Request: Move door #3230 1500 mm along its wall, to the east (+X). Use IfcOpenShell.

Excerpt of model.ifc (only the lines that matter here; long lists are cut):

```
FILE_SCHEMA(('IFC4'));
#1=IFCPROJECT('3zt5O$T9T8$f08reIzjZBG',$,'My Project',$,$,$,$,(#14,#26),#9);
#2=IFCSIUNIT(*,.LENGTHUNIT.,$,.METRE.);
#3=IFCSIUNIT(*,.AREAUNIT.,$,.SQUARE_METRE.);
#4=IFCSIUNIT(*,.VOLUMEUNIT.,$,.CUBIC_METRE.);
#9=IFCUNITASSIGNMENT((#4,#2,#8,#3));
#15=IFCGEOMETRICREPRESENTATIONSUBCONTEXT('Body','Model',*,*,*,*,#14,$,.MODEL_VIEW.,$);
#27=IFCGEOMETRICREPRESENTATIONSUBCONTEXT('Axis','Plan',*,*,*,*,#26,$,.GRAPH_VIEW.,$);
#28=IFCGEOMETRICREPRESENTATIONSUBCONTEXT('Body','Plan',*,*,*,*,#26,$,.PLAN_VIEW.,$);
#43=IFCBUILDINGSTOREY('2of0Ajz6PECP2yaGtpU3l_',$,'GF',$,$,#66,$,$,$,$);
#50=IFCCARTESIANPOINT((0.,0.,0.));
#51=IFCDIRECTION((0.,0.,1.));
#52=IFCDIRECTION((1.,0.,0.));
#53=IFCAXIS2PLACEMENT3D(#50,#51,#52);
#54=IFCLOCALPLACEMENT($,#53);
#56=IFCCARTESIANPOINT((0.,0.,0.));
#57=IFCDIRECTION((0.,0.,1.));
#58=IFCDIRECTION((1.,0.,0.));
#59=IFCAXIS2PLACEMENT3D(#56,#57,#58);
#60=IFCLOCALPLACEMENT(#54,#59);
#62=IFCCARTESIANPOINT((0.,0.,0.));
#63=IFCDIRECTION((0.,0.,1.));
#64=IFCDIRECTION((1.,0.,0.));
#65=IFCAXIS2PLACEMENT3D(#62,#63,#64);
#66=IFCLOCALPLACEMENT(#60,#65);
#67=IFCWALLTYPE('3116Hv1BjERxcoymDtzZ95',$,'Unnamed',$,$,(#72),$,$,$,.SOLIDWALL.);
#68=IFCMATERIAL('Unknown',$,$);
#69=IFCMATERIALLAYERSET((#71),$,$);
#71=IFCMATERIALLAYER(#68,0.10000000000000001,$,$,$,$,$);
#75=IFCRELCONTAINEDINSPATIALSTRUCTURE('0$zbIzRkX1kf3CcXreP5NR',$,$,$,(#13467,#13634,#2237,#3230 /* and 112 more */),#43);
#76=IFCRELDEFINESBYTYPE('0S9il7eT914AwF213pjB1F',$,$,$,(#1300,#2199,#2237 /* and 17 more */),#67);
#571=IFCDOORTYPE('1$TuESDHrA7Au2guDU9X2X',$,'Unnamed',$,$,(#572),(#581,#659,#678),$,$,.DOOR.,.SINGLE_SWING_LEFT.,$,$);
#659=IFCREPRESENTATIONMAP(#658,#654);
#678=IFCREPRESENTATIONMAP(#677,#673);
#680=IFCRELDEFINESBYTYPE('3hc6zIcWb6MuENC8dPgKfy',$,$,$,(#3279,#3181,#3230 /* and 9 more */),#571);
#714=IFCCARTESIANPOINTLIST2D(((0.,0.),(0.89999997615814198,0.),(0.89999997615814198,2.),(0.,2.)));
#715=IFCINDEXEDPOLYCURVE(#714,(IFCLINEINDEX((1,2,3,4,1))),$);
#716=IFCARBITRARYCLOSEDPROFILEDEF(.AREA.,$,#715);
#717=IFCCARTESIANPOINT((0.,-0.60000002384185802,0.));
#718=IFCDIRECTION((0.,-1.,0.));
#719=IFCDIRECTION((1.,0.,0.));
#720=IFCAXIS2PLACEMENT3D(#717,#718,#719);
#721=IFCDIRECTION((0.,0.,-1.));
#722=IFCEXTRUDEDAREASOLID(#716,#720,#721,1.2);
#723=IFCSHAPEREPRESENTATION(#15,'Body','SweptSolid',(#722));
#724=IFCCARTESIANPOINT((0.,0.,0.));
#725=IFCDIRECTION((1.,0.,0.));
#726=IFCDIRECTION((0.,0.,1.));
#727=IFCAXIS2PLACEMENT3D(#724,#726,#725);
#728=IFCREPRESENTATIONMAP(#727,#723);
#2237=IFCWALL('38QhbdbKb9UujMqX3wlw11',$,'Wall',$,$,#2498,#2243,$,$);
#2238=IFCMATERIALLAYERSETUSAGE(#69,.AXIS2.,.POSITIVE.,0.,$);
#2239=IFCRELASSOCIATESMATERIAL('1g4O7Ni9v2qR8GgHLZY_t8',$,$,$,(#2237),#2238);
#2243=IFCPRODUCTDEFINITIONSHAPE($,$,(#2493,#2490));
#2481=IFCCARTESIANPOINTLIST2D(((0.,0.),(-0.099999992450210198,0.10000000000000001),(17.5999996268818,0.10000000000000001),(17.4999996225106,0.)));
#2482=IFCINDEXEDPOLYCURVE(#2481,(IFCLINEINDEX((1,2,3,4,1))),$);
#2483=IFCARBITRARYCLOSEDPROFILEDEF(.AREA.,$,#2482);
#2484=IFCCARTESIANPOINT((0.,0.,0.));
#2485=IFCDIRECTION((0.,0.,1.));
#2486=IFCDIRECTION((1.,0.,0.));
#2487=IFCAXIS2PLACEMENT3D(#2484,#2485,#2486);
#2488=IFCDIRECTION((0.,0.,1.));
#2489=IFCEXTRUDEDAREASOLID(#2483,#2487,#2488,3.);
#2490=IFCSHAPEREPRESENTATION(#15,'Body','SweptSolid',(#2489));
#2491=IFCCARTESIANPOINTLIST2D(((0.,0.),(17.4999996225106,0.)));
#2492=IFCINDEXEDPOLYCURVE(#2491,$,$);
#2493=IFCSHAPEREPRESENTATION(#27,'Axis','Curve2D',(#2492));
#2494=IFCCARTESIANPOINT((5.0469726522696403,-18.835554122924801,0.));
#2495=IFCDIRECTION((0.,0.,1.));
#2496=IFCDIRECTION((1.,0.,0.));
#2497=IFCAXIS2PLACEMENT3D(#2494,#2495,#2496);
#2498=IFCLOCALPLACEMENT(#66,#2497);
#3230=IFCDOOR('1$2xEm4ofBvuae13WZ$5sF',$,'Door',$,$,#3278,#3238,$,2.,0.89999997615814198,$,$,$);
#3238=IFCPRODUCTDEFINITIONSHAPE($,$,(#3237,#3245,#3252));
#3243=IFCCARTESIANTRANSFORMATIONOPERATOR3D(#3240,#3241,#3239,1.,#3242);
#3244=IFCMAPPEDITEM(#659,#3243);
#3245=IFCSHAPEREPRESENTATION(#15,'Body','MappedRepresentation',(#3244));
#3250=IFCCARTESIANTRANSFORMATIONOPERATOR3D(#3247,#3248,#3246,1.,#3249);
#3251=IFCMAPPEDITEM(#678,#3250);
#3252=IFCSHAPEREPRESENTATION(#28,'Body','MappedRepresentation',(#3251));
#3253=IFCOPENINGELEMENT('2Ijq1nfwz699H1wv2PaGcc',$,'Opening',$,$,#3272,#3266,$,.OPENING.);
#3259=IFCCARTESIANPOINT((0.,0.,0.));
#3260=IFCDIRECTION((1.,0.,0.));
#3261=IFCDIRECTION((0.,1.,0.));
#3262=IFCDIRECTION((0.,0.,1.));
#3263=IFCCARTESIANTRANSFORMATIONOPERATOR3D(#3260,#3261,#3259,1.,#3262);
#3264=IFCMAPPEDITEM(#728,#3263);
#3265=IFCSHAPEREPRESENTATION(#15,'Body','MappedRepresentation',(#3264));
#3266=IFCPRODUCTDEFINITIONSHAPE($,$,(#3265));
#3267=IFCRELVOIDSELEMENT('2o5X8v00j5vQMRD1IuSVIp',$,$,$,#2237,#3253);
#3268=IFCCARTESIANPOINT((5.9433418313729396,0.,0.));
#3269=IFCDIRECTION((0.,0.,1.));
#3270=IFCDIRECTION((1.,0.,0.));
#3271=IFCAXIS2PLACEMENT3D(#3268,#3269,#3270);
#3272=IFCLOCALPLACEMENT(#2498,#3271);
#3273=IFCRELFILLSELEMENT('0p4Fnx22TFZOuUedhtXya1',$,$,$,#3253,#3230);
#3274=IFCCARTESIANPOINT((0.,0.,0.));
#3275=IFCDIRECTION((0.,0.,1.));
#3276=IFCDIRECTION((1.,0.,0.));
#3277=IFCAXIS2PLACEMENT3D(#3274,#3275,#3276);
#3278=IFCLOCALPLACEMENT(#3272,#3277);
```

```python
import ifcopenshell
import ifcopenshell.api.geometry
import ifcopenshell.util.placement
import ifcopenshell.util.unit

model = ifcopenshell.open("model.ifc")
unit_scale = ifcopenshell.util.unit.calculate_unit_scale(model)

door = model.by_guid("1$2xEm4ofBvuae13WZ$5sF")
opening = door.FillsVoids[0].RelatingOpeningElement
wall = opening.VoidsElements[0].RelatingBuildingElement

wall_matrix = ifcopenshell.util.placement.get_local_placement(wall.ObjectPlacement)
shift = wall_matrix[:3, 0] * 1.5 / unit_scale
before = ifcopenshell.util.placement.get_local_placement(door.ObjectPlacement)[:3, 3].copy()

# The door is placed relative to its opening, so it follows when the opening moves.
matrix = ifcopenshell.util.placement.get_local_placement(opening.ObjectPlacement)
matrix[:3, 3] += shift
ifcopenshell.api.geometry.edit_object_placement(
    model, product=opening, matrix=matrix, is_si=False, should_transform_children=True
)

after = ifcopenshell.util.placement.get_local_placement(door.ObjectPlacement)[:3, 3]
print("door moved by", (after - before).round(3) + 0.0)

model.write("model_rev.ifc")
```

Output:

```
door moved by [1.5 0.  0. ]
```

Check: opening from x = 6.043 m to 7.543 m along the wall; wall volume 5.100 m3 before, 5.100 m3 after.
